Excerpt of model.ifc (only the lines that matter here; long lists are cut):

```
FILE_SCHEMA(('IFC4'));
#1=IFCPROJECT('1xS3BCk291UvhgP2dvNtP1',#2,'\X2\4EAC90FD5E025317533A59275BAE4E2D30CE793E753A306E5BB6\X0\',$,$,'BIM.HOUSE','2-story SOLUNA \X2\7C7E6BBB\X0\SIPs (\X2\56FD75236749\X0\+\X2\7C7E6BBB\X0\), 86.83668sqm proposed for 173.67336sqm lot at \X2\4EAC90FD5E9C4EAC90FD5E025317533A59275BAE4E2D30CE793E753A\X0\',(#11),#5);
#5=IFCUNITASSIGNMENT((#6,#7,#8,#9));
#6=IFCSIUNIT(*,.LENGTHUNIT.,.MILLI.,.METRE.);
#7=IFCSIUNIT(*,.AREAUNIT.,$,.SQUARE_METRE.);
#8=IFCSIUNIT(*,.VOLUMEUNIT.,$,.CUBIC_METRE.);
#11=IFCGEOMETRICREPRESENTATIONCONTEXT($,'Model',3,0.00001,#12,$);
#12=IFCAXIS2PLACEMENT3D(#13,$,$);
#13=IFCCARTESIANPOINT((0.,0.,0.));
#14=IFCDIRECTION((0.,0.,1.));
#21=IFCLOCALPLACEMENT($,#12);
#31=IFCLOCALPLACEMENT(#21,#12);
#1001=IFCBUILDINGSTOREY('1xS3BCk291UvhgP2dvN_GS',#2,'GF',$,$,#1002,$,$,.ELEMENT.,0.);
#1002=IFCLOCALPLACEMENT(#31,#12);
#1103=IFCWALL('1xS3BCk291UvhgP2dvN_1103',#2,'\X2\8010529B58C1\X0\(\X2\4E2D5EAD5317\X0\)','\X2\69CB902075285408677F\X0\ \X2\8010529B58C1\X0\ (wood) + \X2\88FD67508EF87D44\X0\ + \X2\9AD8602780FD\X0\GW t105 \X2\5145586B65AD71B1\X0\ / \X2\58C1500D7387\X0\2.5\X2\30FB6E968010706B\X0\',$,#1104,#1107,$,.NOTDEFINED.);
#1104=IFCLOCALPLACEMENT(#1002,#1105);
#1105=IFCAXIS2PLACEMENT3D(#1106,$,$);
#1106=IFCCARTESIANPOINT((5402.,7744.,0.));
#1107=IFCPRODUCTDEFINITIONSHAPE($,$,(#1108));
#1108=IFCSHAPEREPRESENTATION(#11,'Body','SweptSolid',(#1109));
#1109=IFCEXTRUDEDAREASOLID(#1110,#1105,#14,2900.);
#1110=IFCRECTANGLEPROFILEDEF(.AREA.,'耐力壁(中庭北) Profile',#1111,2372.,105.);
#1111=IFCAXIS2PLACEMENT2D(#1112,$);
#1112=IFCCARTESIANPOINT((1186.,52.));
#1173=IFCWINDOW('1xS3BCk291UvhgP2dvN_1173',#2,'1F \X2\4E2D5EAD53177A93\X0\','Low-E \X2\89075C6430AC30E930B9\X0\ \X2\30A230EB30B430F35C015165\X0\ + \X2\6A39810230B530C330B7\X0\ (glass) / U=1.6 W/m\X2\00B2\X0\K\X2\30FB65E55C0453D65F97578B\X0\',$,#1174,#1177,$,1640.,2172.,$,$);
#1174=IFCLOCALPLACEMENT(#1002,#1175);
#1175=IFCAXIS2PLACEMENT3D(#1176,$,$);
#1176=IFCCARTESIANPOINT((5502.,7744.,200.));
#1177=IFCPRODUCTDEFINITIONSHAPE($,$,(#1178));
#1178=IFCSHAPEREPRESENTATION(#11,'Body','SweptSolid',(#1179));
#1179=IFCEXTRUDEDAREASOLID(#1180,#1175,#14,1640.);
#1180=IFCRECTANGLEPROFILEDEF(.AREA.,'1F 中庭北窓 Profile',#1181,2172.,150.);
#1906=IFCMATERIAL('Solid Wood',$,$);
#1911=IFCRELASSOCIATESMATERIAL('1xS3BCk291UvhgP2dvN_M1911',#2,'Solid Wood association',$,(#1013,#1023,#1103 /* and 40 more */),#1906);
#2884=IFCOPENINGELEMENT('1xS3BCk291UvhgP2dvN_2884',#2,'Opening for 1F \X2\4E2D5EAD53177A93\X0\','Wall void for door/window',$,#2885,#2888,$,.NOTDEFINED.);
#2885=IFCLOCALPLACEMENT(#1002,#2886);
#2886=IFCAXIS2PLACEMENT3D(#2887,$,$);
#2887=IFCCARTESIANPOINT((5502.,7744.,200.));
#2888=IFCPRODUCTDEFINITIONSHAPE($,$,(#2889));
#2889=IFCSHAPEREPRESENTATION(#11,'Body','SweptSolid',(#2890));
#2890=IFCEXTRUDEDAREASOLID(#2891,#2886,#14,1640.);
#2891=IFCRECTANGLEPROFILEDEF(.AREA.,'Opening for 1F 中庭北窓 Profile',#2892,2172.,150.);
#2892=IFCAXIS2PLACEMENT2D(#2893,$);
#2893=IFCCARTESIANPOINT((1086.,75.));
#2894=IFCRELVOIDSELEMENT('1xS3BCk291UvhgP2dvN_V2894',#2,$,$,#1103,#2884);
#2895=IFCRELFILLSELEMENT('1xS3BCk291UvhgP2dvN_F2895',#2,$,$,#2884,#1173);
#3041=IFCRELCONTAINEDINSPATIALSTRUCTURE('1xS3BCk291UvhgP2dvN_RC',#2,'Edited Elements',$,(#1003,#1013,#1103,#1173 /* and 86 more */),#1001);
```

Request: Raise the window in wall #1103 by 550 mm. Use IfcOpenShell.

```python
import numpy as np
import ifcopenshell
import ifcopenshell.api.geometry
import ifcopenshell.util.placement
import ifcopenshell.util.unit

model = ifcopenshell.open("model.ifc")
unit_scale = ifcopenshell.util.unit.calculate_unit_scale(model)

window = model.by_guid("1xS3BCk291UvhgP2dvN_1173")
opening = window.FillsVoids[0].RelatingOpeningElement
dz = 0.55 / unit_scale

shift = np.array([0.0, 0.0, dz])
# The window is not placed relative to its opening, so move both.
for product in (opening, window):
    matrix = ifcopenshell.util.placement.get_local_placement(product.ObjectPlacement)
    matrix[:3, 3] += shift
    ifcopenshell.api.geometry.edit_object_placement(model, product=product, matrix=matrix, is_si=False)

print(f"moved by {dz * unit_scale:+.3f} m")

model.write("model_updated.ifc")
```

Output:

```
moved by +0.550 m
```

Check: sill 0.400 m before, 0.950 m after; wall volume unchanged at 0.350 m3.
